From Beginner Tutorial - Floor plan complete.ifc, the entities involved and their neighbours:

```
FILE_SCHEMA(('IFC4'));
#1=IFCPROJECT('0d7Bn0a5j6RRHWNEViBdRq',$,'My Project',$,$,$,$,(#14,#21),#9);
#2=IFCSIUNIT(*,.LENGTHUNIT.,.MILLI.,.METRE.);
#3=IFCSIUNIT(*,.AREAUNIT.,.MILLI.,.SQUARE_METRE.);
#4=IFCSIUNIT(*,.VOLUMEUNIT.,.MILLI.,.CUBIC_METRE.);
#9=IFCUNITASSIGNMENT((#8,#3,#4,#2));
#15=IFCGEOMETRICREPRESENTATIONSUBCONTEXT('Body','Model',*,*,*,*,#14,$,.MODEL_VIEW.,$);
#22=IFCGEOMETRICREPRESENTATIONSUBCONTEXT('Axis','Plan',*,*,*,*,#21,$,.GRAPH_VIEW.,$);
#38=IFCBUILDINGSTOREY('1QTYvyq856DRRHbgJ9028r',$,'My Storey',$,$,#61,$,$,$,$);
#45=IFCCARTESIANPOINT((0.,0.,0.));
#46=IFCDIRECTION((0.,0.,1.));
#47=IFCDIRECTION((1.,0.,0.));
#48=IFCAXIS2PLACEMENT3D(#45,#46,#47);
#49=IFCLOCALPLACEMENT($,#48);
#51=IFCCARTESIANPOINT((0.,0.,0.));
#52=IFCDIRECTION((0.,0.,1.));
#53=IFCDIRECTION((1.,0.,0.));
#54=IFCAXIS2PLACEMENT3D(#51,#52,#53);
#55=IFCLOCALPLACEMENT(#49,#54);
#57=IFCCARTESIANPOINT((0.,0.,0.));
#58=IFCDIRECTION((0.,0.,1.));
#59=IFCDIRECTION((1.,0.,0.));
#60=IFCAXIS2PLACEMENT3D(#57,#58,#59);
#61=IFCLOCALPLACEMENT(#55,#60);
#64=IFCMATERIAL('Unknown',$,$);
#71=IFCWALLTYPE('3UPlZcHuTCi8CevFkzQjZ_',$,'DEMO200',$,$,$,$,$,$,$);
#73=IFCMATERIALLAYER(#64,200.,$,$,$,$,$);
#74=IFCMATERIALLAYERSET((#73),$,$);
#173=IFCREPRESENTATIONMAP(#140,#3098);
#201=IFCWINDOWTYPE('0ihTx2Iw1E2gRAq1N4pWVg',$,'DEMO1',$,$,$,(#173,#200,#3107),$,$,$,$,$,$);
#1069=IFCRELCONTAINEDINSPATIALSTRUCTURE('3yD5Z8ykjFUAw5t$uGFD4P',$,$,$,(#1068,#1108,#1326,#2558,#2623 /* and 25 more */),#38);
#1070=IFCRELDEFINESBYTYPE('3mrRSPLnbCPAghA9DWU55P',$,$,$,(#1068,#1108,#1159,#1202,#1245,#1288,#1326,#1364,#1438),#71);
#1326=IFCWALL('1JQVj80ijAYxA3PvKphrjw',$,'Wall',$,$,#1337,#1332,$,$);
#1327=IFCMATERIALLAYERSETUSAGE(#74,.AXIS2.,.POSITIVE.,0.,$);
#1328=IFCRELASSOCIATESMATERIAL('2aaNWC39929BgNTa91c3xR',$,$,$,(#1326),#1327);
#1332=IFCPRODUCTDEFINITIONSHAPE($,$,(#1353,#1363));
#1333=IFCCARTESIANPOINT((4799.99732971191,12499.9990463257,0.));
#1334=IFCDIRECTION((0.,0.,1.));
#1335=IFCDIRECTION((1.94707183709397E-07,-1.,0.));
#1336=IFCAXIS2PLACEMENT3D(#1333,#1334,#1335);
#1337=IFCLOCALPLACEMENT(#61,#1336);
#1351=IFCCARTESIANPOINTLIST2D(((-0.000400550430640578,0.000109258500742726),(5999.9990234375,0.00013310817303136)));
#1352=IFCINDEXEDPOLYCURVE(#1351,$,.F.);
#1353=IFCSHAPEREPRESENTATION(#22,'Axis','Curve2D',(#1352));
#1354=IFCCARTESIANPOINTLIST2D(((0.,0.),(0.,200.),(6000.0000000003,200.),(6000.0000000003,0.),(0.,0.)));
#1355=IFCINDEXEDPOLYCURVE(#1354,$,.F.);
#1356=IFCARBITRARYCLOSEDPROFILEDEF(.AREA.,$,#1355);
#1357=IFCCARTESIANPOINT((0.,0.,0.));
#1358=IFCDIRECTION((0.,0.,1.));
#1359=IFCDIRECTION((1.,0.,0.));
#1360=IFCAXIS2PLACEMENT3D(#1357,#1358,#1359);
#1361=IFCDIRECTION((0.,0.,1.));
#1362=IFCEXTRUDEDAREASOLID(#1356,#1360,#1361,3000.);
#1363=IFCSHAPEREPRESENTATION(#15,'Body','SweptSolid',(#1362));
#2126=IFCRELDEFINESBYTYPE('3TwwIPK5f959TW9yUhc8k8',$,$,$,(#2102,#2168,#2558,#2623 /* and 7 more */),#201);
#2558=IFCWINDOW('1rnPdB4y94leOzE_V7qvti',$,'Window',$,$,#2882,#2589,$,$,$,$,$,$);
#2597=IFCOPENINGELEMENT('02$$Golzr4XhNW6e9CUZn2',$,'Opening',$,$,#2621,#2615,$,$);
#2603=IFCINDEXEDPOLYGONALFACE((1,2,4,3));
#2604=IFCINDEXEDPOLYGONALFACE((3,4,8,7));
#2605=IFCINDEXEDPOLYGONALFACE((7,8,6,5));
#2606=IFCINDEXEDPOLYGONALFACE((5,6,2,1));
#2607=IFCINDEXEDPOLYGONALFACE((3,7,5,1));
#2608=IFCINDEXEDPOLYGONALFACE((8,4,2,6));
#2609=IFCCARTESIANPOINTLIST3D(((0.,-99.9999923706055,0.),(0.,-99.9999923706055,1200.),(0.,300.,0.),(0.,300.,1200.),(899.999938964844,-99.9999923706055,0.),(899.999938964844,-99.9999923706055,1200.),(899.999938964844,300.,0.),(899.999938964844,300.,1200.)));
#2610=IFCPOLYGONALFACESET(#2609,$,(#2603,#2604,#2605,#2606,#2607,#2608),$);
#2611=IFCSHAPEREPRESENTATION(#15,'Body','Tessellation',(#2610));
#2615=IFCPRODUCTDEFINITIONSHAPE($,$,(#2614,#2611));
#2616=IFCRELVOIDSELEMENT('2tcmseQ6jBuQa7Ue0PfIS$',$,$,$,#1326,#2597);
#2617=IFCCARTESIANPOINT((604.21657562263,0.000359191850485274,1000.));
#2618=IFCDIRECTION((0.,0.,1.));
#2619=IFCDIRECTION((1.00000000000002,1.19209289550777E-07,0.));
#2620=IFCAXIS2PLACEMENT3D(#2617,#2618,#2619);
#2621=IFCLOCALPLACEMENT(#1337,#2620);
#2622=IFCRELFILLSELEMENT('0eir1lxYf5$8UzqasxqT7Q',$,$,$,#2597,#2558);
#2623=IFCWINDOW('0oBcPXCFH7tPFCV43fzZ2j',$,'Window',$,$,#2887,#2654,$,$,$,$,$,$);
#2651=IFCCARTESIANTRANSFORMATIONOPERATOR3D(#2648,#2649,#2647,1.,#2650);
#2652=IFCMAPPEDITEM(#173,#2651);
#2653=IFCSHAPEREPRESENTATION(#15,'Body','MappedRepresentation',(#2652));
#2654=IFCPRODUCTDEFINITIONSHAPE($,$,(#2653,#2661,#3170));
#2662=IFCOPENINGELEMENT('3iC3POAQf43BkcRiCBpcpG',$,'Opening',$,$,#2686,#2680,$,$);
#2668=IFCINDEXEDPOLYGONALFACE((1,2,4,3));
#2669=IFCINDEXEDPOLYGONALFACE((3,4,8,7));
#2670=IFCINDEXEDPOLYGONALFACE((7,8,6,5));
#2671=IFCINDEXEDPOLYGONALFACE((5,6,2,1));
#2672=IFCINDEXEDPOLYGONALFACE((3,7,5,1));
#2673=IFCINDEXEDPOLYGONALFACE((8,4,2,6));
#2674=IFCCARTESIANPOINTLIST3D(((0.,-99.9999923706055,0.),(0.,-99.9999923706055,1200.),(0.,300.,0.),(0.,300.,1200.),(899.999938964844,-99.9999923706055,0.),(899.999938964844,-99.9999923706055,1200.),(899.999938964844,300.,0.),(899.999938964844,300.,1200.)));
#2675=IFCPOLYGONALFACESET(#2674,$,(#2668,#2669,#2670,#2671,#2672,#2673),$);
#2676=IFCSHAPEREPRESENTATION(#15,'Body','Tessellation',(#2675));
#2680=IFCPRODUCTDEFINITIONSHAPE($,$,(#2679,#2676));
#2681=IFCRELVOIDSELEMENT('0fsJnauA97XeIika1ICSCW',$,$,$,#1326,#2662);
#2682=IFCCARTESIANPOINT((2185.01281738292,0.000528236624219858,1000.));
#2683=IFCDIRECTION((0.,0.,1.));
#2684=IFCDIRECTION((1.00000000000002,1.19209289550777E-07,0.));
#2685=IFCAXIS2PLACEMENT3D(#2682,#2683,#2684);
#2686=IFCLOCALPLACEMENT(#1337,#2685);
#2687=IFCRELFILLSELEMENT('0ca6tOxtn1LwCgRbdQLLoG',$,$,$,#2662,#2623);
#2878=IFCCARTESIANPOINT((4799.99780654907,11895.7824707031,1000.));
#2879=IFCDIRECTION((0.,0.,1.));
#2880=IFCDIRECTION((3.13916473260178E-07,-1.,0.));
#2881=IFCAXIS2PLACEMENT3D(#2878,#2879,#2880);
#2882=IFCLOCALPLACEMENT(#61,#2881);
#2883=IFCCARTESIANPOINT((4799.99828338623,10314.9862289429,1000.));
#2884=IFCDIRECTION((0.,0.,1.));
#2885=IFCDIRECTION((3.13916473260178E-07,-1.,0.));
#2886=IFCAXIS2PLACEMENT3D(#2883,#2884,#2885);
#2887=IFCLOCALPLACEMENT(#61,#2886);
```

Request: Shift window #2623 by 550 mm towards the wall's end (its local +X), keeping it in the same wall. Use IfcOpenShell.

```python
import ifcopenshell
import ifcopenshell.api.geometry
import ifcopenshell.util.placement
import ifcopenshell.util.unit

model = ifcopenshell.open("Beginner Tutorial - Floor plan complete.ifc")
unit_scale = ifcopenshell.util.unit.calculate_unit_scale(model)

window = model.by_guid("0oBcPXCFH7tPFCV43fzZ2j")
opening = window.FillsVoids[0].RelatingOpeningElement
wall = opening.VoidsElements[0].RelatingBuildingElement

wall_matrix = ifcopenshell.util.placement.get_local_placement(wall.ObjectPlacement)
shift = wall_matrix[:3, 0] * 0.55 / unit_scale
before = ifcopenshell.util.placement.get_local_placement(window.ObjectPlacement)[:3, 3].copy()

# The window is not placed relative to its opening, so move both.
for product in (opening, window):
    matrix = ifcopenshell.util.placement.get_local_placement(product.ObjectPlacement)
    matrix[:3, 3] += shift
    ifcopenshell.api.geometry.edit_object_placement(model, product=product, matrix=matrix, is_si=False)

after = ifcopenshell.util.placement.get_local_placement(window.ObjectPlacement)[:3, 3]
print("window moved by", (after - before).round(3) + 0.0)

model.write("Beginner Tutorial - Floor plan complete-out.ifc")
```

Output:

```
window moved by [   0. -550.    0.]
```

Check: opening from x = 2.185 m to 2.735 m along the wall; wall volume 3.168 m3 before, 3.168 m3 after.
